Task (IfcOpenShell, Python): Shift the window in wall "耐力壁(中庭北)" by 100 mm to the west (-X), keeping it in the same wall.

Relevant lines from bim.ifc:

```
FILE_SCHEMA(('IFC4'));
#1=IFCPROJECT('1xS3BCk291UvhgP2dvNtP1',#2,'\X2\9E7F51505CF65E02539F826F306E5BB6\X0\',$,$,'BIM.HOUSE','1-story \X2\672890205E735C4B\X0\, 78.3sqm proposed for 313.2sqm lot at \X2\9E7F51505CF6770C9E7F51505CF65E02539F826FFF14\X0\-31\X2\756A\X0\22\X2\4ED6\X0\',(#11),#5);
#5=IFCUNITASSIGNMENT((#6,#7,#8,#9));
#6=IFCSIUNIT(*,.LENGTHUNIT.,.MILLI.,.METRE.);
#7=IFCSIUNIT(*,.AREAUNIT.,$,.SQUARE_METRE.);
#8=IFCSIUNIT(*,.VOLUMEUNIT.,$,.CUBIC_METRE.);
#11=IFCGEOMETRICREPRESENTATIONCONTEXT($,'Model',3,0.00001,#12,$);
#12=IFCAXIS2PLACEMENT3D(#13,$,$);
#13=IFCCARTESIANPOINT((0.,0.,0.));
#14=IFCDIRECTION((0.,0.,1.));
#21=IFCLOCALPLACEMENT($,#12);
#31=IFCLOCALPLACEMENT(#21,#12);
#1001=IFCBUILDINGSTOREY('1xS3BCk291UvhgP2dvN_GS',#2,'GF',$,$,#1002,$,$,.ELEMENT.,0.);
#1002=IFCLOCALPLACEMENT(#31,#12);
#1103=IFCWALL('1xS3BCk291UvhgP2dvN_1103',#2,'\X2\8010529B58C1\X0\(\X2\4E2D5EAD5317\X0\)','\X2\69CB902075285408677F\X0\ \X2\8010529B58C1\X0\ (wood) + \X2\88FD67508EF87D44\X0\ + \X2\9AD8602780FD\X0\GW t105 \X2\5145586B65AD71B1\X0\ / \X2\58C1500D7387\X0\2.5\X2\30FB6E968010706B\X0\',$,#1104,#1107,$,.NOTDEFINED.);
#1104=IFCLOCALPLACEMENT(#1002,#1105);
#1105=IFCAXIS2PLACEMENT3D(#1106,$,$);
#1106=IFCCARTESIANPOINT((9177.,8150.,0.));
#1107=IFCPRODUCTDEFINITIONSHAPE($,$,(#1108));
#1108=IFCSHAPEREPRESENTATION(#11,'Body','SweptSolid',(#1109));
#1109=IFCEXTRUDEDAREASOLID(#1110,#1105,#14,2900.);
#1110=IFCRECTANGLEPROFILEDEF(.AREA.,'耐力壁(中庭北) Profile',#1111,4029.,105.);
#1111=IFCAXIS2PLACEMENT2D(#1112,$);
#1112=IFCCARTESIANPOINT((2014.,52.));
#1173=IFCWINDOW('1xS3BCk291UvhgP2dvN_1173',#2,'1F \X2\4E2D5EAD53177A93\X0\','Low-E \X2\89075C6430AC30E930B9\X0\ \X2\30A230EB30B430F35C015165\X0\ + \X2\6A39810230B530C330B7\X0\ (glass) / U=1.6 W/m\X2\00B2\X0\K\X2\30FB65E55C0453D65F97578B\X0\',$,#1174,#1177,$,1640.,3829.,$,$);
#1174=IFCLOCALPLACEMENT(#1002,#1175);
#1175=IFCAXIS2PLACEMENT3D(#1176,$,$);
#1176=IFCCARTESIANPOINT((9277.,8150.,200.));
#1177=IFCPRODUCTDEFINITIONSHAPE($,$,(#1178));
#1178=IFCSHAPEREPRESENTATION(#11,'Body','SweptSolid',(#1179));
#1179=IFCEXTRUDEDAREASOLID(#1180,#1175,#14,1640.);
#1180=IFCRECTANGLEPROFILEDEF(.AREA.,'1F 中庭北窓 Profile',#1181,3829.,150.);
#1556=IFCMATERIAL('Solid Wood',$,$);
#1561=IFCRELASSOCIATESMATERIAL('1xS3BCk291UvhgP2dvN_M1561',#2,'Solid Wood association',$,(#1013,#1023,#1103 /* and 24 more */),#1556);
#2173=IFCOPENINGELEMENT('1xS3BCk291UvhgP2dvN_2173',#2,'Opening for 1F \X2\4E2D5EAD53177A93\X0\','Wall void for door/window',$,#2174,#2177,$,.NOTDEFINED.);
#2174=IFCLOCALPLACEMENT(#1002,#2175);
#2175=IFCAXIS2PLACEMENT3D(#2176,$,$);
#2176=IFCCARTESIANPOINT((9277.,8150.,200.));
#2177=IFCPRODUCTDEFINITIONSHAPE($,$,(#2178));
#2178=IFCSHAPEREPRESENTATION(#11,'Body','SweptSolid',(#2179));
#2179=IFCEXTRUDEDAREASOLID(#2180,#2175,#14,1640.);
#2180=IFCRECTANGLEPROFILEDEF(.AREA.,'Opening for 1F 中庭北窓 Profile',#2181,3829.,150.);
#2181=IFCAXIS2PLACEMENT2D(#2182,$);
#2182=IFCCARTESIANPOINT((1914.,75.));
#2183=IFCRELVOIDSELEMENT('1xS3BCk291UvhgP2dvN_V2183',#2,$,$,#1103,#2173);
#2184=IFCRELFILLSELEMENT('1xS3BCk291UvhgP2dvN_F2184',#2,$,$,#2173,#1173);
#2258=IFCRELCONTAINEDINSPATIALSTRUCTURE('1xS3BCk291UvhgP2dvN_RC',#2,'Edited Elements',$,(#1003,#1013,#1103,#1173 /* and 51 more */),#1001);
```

```python
import ifcopenshell
import ifcopenshell.api.geometry
import ifcopenshell.util.placement
import ifcopenshell.util.unit

model = ifcopenshell.open("bim.ifc")
unit_scale = ifcopenshell.util.unit.calculate_unit_scale(model)

window = model.by_guid("1xS3BCk291UvhgP2dvN_1173")
opening = window.FillsVoids[0].RelatingOpeningElement
wall = opening.VoidsElements[0].RelatingBuildingElement

wall_matrix = ifcopenshell.util.placement.get_local_placement(wall.ObjectPlacement)
shift = wall_matrix[:3, 0] * -0.1 / unit_scale
before = ifcopenshell.util.placement.get_local_placement(window.ObjectPlacement)[:3, 3].copy()

# The window is not placed relative to its opening, so move both.
for product in (opening, window):
    matrix = ifcopenshell.util.placement.get_local_placement(product.ObjectPlacement)
    matrix[:3, 3] += shift
    ifcopenshell.api.geometry.edit_object_placement(model, product=product, matrix=matrix, is_si=False)

after = ifcopenshell.util.placement.get_local_placement(window.ObjectPlacement)[:3, 3]
print("window moved by", (after - before).round(3) + 0.0)

model.write("bim-out.ifc")
```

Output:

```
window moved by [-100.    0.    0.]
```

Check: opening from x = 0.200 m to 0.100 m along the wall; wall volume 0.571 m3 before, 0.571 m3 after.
